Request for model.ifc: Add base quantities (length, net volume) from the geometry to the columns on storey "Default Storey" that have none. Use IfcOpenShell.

First a look at what the model holds.

```python
import ifcopenshell
import ifcopenshell.util.element
import ifcopenshell.util.unit

model = ifcopenshell.open("model.ifc")
print(model.schema)
for unit_type in ("LENGTHUNIT", "AREAUNIT", "VOLUMEUNIT"):
    print(unit_type, ifcopenshell.util.unit.calculate_unit_scale(model, unit_type))
storey = next(s for s in model.by_type("IfcBuildingStorey") if s.Name == "Default Storey")
columns = [e for e in ifcopenshell.util.element.get_decomposition(storey) if e.is_a("IfcColumn")]
for e in sorted(columns, key=lambda e: e.id()):
    print(e.id(), e.is_a(), e.Name, list(ifcopenshell.util.element.get_psets(e, qtos_only=True)), sep=" | ")
```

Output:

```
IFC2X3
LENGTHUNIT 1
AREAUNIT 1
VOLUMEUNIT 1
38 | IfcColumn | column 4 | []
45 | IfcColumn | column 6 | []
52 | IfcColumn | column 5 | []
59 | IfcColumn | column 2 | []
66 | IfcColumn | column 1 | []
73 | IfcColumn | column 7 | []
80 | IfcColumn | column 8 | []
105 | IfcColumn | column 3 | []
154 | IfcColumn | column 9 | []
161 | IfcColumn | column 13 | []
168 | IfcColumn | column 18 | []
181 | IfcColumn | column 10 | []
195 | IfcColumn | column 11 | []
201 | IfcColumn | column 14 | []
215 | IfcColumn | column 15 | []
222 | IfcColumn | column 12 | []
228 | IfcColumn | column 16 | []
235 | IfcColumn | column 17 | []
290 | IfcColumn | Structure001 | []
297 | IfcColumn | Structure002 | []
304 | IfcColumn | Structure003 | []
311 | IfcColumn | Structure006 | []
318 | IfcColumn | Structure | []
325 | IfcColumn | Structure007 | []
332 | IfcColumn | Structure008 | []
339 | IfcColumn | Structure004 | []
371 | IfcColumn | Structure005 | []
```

```python
import ifcopenshell
import ifcopenshell.api.pset
import ifcopenshell.geom
import ifcopenshell.util.element
import ifcopenshell.util.shape
import ifcopenshell.util.unit

model = ifcopenshell.open("model.ifc")
unit_scale = ifcopenshell.util.unit.calculate_unit_scale(model)
volume_scale = ifcopenshell.util.unit.calculate_unit_scale(model, "VOLUMEUNIT")
settings = ifcopenshell.geom.settings()

storey = next(s for s in model.by_type("IfcBuildingStorey") if s.Name == "Default Storey")
columns = [e for e in ifcopenshell.util.element.get_decomposition(storey) if e.is_a("IfcColumn")]

for e in sorted(columns, key=lambda e: e.id()):
    if ifcopenshell.util.element.get_psets(e, qtos_only=True, should_inherit=False):
        continue
    # Geometry comes back in metres, in the element's own axes.
    shape = ifcopenshell.geom.create_shape(settings, e)
    values = {
        "Length": ifcopenshell.util.shape.get_z(shape.geometry) / unit_scale,
        "NetVolume": ifcopenshell.util.shape.get_volume(shape.geometry) / volume_scale,
    }
    qto = ifcopenshell.api.pset.add_qto(model, product=e, name="BaseQuantities")
    ifcopenshell.api.pset.edit_qto(model, qto=qto, properties=values)
    print(e.id(), {k: round(v, 3) for k, v in values.items()})

model.write("model_edited.ifc")
```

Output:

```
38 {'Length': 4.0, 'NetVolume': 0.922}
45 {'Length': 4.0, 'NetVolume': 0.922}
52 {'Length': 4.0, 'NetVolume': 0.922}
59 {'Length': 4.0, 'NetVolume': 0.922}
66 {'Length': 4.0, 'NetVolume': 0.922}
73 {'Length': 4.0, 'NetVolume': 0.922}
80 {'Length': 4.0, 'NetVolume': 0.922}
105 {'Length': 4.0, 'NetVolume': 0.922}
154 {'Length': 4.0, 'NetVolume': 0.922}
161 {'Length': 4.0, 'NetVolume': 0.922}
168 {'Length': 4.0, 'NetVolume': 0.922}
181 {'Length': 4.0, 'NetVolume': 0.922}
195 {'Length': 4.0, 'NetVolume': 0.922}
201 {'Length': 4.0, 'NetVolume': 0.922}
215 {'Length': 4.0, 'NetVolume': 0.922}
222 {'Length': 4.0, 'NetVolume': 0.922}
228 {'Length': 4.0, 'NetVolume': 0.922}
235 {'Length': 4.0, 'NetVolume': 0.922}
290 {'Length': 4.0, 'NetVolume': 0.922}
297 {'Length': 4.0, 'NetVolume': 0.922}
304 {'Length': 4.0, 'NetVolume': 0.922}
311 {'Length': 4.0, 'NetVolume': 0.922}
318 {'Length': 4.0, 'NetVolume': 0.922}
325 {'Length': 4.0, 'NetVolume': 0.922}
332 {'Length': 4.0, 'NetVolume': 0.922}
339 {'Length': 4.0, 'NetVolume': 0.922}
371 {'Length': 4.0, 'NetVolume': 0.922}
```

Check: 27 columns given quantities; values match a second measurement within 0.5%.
